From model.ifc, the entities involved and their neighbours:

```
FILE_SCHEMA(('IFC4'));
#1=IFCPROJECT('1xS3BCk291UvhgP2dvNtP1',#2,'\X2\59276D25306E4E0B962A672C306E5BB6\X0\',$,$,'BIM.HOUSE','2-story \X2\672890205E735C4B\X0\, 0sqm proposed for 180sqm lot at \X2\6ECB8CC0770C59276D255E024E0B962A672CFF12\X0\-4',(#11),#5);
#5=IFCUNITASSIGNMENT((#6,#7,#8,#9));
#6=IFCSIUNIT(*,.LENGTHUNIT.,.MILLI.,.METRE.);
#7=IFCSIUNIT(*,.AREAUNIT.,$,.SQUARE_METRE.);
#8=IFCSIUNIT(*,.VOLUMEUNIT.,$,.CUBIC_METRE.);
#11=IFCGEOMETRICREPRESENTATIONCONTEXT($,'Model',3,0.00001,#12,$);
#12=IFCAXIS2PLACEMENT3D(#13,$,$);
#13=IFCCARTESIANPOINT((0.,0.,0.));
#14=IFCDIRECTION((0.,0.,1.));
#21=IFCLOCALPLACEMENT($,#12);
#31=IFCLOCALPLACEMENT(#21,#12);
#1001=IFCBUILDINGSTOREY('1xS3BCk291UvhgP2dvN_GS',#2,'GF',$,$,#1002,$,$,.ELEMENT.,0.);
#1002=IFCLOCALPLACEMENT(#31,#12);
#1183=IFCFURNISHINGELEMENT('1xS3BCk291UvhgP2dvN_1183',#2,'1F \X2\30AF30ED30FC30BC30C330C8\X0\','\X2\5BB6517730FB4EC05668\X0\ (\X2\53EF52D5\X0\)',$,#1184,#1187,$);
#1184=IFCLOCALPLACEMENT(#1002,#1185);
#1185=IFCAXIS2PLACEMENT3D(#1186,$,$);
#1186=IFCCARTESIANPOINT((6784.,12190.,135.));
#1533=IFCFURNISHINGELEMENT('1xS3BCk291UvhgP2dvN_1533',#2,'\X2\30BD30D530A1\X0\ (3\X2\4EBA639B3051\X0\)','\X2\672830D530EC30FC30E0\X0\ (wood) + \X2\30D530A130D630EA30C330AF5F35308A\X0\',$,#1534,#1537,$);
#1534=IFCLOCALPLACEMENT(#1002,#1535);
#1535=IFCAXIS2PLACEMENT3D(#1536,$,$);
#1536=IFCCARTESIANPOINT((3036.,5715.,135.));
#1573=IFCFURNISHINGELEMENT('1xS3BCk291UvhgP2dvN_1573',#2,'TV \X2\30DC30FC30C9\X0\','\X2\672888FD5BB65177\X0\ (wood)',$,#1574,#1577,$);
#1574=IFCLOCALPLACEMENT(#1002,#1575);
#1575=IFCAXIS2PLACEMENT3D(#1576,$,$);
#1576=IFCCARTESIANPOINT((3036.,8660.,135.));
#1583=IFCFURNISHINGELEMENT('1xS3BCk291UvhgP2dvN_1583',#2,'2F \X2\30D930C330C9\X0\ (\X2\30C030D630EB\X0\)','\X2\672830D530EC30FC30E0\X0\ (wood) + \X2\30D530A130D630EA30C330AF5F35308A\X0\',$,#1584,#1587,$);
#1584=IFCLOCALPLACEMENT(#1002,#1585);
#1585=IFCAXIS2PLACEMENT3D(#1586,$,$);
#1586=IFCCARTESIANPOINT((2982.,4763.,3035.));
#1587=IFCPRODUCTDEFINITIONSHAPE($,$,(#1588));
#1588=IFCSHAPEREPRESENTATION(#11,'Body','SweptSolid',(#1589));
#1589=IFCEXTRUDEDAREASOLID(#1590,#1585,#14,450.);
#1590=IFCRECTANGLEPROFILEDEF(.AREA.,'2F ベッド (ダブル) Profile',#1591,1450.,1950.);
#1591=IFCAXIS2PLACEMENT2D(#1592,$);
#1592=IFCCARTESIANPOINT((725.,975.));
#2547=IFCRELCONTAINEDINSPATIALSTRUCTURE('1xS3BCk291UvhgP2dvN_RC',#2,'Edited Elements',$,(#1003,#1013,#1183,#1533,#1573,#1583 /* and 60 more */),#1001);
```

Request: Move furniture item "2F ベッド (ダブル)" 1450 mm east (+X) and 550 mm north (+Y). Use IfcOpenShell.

```python
import ifcopenshell
import ifcopenshell.api.geometry
import ifcopenshell.util.placement

model = ifcopenshell.open("model.ifc")

item = model.by_guid("1xS3BCk291UvhgP2dvN_1583")
matrix = ifcopenshell.util.placement.get_local_placement(item.ObjectPlacement)
matrix[0, 3] += 1450.0
matrix[1, 3] += 550.0
ifcopenshell.api.geometry.edit_object_placement(model, product=item, matrix=matrix, is_si=False)

print(ifcopenshell.util.placement.get_local_placement(item.ObjectPlacement).round(3) + 0.0)

model.write("model_updated.ifc")
```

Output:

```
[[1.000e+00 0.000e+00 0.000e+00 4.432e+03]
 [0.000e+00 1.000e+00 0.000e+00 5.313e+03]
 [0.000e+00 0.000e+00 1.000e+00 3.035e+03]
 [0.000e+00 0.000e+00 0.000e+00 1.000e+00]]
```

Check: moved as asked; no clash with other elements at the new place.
